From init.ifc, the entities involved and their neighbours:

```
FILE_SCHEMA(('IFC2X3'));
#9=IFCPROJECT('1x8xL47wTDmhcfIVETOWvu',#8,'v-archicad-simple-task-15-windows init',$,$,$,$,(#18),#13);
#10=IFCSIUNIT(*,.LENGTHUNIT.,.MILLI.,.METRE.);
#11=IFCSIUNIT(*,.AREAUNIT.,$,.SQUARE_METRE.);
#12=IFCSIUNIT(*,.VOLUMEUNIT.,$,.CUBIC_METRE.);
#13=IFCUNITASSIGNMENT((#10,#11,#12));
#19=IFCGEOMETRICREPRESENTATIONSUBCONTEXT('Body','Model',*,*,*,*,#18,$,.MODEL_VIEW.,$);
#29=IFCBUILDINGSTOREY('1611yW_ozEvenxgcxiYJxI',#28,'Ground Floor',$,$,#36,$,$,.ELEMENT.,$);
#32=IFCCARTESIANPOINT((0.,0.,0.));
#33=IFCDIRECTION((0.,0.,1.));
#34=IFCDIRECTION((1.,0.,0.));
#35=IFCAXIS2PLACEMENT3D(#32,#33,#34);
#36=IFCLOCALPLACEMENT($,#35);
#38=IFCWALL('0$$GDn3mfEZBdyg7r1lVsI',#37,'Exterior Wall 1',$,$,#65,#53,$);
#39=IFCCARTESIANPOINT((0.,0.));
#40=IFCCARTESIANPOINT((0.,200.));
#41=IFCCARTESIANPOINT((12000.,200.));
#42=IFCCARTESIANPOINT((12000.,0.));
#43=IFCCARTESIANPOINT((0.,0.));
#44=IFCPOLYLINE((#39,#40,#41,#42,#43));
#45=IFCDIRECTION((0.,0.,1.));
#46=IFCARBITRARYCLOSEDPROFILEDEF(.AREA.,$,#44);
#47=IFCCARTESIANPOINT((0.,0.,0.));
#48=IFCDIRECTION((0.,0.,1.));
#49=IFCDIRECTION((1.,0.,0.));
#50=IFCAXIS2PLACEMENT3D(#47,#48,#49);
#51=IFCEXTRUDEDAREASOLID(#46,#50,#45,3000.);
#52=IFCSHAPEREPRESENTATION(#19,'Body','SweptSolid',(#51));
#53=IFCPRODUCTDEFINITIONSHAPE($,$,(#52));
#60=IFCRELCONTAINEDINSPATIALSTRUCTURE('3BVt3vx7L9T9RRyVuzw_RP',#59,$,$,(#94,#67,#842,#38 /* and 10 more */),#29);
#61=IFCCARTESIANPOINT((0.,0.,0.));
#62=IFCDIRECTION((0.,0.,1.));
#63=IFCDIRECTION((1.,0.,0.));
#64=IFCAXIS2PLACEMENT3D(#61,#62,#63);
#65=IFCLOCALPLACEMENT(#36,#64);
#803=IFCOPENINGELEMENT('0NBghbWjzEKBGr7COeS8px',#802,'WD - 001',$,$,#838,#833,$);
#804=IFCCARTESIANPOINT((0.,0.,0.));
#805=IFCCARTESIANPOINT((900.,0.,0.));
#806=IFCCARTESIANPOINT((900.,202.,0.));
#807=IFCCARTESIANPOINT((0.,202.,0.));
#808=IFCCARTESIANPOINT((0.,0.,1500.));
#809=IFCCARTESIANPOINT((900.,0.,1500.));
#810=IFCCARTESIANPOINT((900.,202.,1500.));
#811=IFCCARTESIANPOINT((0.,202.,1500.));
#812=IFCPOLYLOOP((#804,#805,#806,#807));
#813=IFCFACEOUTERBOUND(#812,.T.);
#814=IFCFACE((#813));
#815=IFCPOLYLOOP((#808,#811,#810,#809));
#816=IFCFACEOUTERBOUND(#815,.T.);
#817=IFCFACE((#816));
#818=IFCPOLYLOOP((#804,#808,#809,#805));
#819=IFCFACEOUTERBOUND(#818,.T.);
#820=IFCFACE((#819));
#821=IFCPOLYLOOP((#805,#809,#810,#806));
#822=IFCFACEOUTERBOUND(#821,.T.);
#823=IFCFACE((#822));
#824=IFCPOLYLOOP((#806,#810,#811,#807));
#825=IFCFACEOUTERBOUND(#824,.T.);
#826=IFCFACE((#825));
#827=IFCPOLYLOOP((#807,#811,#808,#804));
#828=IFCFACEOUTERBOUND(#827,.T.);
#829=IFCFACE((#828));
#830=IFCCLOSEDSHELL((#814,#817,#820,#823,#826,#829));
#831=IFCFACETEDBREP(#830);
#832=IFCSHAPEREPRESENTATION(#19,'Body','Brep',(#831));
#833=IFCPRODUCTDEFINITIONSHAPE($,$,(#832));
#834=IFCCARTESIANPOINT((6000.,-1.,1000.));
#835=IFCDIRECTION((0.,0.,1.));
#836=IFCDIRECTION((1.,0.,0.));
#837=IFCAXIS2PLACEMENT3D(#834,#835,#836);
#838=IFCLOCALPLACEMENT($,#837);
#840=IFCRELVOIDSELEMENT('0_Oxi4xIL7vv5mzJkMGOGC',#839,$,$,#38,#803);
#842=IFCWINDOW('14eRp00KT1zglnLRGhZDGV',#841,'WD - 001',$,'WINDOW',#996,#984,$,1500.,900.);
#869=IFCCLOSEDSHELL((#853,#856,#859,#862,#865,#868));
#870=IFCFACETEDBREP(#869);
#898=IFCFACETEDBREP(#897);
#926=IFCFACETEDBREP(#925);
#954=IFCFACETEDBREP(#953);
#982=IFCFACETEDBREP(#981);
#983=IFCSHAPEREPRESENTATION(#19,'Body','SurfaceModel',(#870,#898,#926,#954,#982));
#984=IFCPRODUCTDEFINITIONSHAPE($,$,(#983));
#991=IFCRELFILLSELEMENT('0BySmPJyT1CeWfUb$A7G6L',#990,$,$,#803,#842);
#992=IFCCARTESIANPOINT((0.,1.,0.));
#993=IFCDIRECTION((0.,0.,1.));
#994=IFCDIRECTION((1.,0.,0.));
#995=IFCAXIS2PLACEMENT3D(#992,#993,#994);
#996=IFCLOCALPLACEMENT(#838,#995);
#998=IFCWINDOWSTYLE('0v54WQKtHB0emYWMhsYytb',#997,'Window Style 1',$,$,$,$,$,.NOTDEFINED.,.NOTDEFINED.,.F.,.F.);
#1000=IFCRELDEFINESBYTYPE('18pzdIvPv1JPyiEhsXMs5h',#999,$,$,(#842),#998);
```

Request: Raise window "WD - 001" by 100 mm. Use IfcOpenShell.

```python
import numpy as np
import ifcopenshell
import ifcopenshell.api.geometry
import ifcopenshell.util.placement
import ifcopenshell.util.unit

model = ifcopenshell.open("init.ifc")
unit_scale = ifcopenshell.util.unit.calculate_unit_scale(model)

window = model.by_guid("14eRp00KT1zglnLRGhZDGV")
opening = window.FillsVoids[0].RelatingOpeningElement
dz = 0.1 / unit_scale

shift = np.array([0.0, 0.0, dz])
# The window is placed relative to its opening, so it follows when the opening moves.
matrix = ifcopenshell.util.placement.get_local_placement(opening.ObjectPlacement)
matrix[:3, 3] += shift
ifcopenshell.api.geometry.edit_object_placement(
    model, product=opening, matrix=matrix, is_si=False, should_transform_children=True
)

print(f"moved by {dz * unit_scale:+.3f} m")

model.write("init_rev.ifc")
```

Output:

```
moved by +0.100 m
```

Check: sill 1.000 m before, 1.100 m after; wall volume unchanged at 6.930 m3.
